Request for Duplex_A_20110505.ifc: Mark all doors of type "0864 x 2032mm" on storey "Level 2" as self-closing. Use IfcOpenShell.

First a look at what the model holds.

```python
import ifcopenshell
import ifcopenshell.util.element

model = ifcopenshell.open("Duplex_A_20110505.ifc")
print(model.schema)
storey = next(s for s in model.by_type("IfcBuildingStorey") if s.Name == "Level 2")
doors = [e for e in ifcopenshell.util.element.get_decomposition(storey) if e.is_a("IfcDoor")]
seen = {}
for e in doors:
    element_type = ifcopenshell.util.element.get_type(e)
    key = (element_type.Name if element_type != e and element_type else None, ifcopenshell.util.element.get_pset(e, "Pset_DoorCommon", "SelfClosing"))
    seen[key] = seen.get(key, 0) + 1
for (name, value), count in sorted(seen.items(), key=str):
    print(count, "x", name, "|", value)
```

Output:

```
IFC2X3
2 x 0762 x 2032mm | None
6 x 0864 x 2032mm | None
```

```python
import ifcopenshell
import ifcopenshell.api.pset
import ifcopenshell.util.element

model = ifcopenshell.open("Duplex_A_20110505.ifc")

storey = next(s for s in model.by_type("IfcBuildingStorey") if s.Name == "Level 2")
doors = [e for e in ifcopenshell.util.element.get_decomposition(storey) if e.is_a("IfcDoor")]

count = 0
for e in doors:
    element_type = ifcopenshell.util.element.get_type(e)
    if element_type in (None, e) or element_type.Name != "0864 x 2032mm":
        continue
    # add_pset returns the element's existing set when there is one.
    pset = ifcopenshell.api.pset.add_pset(model, product=e, name="Pset_DoorCommon")
    ifcopenshell.api.pset.edit_pset(model, pset=pset, properties={"SelfClosing": True})
    count += 1

print(count, "doors updated")

model.write("Duplex_A_20110505_updated.ifc")
```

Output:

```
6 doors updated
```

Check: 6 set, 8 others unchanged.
